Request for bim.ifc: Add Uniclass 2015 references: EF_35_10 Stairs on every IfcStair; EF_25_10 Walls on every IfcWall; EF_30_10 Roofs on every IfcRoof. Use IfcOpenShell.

First a look at what the model holds.

```python
import ifcopenshell

model = ifcopenshell.open("bim.ifc")
print(model.schema)
print("classifications:", [c.Name for c in model.by_type("IfcClassification")])
for ifc_class in ("IfcDoor", "IfcRoof", "IfcStair", "IfcWall", "IfcWindow"):
    print(ifc_class, len(model.by_type(ifc_class)))
```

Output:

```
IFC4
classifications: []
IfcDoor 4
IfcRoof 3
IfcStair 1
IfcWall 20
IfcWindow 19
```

```python
import ifcopenshell
import ifcopenshell.api.classification

model = ifcopenshell.open("bim.ifc")

system = ifcopenshell.api.classification.add_classification(model, classification="Uniclass 2015")

codes = {
    "IfcStair": ("EF_35_10", "Stairs"),
    "IfcWall": ("EF_25_10", "Walls"),
    "IfcRoof": ("EF_30_10", "Roofs"),
}
for ifc_class, (code, name) in codes.items():
    products = model.by_type(ifc_class)
    ifcopenshell.api.classification.add_reference(
        model, products=products, classification=system, identification=code, name=name
    )
    print(code, len(products))

model.write("bim_updated.ifc")
```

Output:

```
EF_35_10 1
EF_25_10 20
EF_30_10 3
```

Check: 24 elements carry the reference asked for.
